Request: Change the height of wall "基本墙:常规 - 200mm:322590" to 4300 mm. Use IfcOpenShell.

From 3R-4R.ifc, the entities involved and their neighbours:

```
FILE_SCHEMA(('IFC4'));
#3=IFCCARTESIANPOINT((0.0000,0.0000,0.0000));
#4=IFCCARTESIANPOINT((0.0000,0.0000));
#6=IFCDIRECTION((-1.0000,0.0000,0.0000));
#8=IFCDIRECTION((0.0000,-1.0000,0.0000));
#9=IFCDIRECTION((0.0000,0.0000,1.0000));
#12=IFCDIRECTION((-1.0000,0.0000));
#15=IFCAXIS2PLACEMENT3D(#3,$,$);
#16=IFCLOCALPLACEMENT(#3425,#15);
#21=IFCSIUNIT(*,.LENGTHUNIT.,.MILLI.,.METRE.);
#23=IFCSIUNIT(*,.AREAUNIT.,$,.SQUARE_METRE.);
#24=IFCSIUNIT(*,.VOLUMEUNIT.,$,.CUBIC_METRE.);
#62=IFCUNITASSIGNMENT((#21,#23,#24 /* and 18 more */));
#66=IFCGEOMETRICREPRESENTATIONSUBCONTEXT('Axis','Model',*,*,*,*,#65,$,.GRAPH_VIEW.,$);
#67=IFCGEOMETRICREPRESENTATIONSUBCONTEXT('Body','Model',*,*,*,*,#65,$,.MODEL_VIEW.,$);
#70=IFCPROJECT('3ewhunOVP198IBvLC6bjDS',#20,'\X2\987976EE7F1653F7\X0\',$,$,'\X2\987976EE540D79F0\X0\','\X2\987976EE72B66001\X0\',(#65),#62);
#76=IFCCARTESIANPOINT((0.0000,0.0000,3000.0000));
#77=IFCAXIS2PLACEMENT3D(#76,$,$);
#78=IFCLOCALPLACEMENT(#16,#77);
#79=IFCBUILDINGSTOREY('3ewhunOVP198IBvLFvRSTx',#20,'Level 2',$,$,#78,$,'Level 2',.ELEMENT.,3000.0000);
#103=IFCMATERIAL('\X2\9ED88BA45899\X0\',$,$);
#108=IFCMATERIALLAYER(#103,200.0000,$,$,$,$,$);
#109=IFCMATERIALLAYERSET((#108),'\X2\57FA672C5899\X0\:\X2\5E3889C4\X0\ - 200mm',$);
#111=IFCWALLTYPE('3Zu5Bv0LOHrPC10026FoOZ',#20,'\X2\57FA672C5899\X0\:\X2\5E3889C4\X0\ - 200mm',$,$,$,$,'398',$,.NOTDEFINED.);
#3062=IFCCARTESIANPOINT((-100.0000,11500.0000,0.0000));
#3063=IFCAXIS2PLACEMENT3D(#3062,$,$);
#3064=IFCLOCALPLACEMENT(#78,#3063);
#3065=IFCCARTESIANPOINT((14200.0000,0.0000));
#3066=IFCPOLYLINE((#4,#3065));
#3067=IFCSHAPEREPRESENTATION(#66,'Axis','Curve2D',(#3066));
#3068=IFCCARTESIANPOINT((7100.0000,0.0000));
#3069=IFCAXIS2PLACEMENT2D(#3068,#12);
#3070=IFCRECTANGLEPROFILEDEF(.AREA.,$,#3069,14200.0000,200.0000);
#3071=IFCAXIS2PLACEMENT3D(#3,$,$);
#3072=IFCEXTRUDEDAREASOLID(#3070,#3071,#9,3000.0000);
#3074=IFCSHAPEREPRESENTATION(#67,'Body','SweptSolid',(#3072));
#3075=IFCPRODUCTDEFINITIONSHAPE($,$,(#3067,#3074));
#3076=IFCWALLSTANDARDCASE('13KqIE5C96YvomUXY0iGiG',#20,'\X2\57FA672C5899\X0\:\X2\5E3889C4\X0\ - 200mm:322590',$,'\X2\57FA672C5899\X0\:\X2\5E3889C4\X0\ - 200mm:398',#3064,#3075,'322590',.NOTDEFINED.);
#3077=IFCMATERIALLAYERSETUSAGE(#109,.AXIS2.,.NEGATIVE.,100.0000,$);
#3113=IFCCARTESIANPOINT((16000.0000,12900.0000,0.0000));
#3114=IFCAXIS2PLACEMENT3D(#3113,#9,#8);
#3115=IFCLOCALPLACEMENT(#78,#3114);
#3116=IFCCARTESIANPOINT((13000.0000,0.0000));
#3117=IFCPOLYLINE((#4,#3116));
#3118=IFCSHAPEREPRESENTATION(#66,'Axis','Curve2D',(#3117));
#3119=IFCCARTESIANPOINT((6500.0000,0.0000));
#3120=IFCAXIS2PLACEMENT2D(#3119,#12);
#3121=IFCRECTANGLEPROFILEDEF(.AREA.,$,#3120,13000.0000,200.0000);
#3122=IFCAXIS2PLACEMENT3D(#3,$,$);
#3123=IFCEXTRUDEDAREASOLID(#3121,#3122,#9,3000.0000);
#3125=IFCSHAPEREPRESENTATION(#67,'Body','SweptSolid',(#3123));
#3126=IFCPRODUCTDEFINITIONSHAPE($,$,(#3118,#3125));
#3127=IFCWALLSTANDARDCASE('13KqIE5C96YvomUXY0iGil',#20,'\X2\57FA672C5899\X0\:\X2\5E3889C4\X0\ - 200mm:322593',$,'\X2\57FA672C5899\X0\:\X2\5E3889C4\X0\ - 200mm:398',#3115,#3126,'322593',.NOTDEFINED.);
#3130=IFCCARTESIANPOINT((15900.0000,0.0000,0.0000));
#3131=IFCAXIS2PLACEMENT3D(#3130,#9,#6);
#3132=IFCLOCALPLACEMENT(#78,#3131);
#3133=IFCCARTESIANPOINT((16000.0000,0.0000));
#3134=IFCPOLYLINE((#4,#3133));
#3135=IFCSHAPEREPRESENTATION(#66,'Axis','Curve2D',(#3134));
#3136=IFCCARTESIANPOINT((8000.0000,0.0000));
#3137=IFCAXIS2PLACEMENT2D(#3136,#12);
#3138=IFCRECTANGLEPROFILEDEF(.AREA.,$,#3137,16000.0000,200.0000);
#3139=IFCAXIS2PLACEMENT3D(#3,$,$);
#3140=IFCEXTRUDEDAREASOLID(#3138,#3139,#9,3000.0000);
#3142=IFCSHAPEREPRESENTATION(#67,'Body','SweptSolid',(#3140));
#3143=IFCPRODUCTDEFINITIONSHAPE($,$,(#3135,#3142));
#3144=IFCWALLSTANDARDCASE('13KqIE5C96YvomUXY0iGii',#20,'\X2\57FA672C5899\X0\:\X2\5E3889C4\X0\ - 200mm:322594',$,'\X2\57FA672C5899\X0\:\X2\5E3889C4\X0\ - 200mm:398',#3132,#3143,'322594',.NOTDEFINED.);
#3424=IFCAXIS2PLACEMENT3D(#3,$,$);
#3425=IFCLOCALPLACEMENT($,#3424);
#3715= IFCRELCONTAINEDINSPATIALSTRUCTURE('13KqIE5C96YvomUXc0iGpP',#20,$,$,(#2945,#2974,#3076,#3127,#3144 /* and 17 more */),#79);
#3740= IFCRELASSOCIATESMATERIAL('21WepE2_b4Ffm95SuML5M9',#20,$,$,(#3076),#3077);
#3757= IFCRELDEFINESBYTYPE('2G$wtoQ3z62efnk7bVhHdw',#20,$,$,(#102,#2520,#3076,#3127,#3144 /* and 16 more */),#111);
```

```python
import ifcopenshell
import ifcopenshell.geom
import ifcopenshell.util.representation
import ifcopenshell.util.shape
import ifcopenshell.util.unit

model = ifcopenshell.open("3R-4R.ifc")
unit_scale = ifcopenshell.util.unit.calculate_unit_scale(model)
settings = ifcopenshell.geom.settings()


def volume(element):
    """Net volume in cubic metres, openings subtracted."""
    shape = ifcopenshell.geom.create_shape(settings, element)
    return ifcopenshell.util.shape.get_volume(shape.geometry)


wall = model.by_guid("13KqIE5C96YvomUXY0iGiG")
before = volume(wall)

body = ifcopenshell.util.representation.get_representation(wall, "Model", "Body")
solid = body.Items[0]
old_height = solid.Depth
solid.Depth = 4.3 / unit_scale
after = volume(wall)

print(f"height {old_height:g} -> {solid.Depth:g}, volume {before:.3f} -> {after:.3f} m3")

model.write("3R-4R_updated.ifc")
```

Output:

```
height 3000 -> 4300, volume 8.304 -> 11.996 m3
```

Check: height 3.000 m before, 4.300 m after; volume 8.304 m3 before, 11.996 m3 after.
